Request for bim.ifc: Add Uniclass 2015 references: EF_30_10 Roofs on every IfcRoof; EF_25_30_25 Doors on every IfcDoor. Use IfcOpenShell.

First a look at what the model holds.

```python
import ifcopenshell

model = ifcopenshell.open("bim.ifc")
print(model.schema)
print("classifications:", [c.Name for c in model.by_type("IfcClassification")])
for ifc_class in ("IfcDoor", "IfcRoof", "IfcStair", "IfcWall", "IfcWindow"):
    print(ifc_class, len(model.by_type(ifc_class)))
```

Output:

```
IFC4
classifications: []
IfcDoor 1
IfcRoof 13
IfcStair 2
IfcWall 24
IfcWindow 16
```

```python
import ifcopenshell
import ifcopenshell.api.classification

model = ifcopenshell.open("bim.ifc")

system = ifcopenshell.api.classification.add_classification(model, classification="Uniclass 2015")

codes = {
    "IfcRoof": ("EF_30_10", "Roofs"),
    "IfcDoor": ("EF_25_30_25", "Doors"),
}
for ifc_class, (code, name) in codes.items():
    products = model.by_type(ifc_class)
    ifcopenshell.api.classification.add_reference(
        model, products=products, classification=system, identification=code, name=name
    )
    print(code, len(products))

model.write("bim_rev.ifc")
```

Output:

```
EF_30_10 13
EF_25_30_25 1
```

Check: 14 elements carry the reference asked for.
